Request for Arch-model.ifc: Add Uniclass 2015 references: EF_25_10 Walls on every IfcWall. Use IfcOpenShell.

First a look at what the model holds.

```python
import ifcopenshell

model = ifcopenshell.open("Arch-model.ifc")
print(model.schema)
print("classifications:", [c.Name for c in model.by_type("IfcClassification")])
for ifc_class in ("IfcDoor", "IfcRoof", "IfcStair", "IfcWall", "IfcWindow"):
    print(ifc_class, len(model.by_type(ifc_class)))
```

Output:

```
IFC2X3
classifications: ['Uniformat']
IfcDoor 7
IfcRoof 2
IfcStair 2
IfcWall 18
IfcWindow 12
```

```python
import ifcopenshell
import ifcopenshell.api.classification

model = ifcopenshell.open("Arch-model.ifc")

# IFC2X3 requires Source and Edition and has no link from the project to the system.
system = model.create_entity("IfcClassification", Source="NBS", Edition="2015", Name="Uniclass 2015")

codes = {
    "IfcWall": ("EF_25_10", "Walls"),
}
for ifc_class, (code, name) in codes.items():
    products = model.by_type(ifc_class)
    ifcopenshell.api.classification.add_reference(
        model, products=products, classification=system, identification=code, name=name
    )
    print(code, len(products))

model.write("Arch-model_v2.ifc")
```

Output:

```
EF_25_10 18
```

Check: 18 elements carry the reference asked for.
